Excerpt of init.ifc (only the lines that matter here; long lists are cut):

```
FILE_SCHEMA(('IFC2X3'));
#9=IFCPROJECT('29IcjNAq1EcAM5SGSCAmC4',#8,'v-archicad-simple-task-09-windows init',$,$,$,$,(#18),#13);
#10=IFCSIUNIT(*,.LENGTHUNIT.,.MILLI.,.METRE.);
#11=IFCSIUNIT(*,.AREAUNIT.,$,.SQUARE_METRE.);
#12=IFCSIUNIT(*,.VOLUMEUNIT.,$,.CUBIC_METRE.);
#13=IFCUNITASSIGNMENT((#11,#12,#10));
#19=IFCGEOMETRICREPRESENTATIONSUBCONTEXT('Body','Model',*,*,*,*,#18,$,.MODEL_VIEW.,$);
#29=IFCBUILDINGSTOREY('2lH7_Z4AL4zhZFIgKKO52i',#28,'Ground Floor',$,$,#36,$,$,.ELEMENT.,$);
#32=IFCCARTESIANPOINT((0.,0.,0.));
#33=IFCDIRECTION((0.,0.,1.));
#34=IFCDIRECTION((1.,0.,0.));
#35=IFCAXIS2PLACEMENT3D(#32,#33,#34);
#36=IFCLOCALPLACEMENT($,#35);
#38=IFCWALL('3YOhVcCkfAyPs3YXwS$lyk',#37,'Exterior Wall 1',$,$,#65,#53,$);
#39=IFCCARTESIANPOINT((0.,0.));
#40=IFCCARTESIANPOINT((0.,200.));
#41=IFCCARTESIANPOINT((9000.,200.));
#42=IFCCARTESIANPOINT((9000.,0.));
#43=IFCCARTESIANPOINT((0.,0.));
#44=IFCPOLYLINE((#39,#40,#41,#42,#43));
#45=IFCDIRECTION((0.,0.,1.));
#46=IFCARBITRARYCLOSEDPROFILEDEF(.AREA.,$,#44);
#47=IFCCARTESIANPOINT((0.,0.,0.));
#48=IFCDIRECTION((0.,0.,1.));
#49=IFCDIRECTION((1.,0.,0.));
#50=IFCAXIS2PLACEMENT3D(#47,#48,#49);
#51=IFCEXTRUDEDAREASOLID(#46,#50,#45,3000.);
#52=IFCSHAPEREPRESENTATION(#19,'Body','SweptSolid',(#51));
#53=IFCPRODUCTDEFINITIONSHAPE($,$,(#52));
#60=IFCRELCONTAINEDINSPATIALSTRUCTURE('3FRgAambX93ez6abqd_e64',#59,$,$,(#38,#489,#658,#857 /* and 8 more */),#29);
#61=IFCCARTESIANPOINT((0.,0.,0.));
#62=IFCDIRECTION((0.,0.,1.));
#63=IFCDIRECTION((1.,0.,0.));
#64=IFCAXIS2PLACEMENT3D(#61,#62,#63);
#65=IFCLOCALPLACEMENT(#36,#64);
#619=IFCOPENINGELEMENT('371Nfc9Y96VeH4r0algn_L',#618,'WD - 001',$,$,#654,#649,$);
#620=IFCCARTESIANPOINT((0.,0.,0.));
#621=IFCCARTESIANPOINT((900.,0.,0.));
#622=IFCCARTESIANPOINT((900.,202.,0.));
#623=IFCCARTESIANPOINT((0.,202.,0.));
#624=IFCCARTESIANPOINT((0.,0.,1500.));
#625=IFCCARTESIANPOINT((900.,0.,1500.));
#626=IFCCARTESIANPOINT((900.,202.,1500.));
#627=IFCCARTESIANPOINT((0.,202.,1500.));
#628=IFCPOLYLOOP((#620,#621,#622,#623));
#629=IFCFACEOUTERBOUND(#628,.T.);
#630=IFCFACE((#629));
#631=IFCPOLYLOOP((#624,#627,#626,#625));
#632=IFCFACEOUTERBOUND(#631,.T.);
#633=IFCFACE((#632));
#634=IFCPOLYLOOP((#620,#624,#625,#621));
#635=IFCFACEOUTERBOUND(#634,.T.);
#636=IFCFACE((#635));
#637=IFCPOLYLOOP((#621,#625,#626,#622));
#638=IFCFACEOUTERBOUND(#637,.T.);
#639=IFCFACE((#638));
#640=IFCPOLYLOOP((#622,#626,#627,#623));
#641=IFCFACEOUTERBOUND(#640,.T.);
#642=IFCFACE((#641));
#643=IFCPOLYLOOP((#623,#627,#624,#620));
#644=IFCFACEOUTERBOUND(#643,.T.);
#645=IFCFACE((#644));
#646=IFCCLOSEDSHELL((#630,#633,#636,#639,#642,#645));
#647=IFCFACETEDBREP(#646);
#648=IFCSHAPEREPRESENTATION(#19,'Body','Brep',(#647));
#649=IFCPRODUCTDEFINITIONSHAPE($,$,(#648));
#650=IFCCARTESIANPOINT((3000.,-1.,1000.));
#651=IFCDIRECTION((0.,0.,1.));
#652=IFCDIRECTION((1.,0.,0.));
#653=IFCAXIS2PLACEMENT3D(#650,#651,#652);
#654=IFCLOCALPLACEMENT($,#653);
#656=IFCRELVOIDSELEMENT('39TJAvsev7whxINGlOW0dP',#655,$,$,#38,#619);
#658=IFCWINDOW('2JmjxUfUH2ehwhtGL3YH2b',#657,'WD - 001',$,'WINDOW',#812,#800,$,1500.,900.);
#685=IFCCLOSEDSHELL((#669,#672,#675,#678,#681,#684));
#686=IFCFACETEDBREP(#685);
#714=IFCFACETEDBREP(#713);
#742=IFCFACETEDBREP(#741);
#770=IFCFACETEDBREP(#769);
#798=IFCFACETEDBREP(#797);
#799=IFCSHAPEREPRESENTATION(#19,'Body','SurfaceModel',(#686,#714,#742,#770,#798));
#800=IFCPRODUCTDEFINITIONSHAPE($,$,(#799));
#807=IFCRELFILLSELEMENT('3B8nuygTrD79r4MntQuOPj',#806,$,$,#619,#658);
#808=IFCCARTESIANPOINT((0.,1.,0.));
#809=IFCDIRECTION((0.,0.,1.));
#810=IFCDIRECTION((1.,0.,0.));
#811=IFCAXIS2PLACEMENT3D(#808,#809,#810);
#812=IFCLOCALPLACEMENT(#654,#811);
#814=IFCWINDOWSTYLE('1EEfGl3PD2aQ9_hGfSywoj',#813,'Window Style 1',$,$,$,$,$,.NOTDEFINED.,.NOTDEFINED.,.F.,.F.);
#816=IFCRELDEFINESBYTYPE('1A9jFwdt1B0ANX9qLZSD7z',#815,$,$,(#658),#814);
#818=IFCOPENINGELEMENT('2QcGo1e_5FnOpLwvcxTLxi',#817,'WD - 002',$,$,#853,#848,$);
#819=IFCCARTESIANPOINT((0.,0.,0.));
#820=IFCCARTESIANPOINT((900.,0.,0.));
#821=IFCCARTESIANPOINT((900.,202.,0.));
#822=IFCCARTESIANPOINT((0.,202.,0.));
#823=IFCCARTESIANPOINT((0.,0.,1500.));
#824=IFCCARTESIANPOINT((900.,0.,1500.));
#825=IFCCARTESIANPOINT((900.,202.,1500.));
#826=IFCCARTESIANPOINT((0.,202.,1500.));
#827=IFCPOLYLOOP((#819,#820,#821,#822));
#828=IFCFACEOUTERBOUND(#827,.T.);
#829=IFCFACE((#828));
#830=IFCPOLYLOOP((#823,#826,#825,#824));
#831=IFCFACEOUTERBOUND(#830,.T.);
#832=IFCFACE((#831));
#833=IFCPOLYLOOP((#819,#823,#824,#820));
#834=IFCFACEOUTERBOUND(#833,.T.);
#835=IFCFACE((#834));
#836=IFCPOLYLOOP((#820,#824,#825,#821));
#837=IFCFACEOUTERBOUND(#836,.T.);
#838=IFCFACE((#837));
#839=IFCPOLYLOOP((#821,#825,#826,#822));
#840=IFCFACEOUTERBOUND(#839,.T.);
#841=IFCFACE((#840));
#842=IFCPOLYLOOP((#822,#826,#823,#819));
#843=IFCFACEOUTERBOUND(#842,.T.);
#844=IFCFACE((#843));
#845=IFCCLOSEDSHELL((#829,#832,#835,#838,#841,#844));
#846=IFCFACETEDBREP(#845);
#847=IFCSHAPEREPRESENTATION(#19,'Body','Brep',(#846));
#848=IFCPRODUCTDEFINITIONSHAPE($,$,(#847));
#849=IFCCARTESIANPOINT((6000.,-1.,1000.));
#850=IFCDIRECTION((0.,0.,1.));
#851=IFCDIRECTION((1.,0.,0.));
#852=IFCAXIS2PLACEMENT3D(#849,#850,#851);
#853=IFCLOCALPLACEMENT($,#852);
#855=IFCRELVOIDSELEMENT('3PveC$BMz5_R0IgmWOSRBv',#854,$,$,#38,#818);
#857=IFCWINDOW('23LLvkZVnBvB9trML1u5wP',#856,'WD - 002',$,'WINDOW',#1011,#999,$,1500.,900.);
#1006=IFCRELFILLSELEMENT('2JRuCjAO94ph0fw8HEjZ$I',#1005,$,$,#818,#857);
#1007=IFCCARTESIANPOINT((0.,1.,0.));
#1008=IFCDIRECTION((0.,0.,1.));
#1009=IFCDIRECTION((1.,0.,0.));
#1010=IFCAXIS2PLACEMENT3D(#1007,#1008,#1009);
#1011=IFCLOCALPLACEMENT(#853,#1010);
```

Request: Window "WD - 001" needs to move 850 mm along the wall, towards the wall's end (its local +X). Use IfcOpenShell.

```python
import ifcopenshell
import ifcopenshell.api.geometry
import ifcopenshell.util.placement

model = ifcopenshell.open("init.ifc")

window = model.by_guid("2JmjxUfUH2ehwhtGL3YH2b")
opening = window.FillsVoids[0].RelatingOpeningElement
wall = opening.VoidsElements[0].RelatingBuildingElement

wall_matrix = ifcopenshell.util.placement.get_local_placement(wall.ObjectPlacement)
shift = wall_matrix[:3, 0] * 850.0
before = ifcopenshell.util.placement.get_local_placement(window.ObjectPlacement)[:3, 3].copy()

# The window is placed relative to its opening, so it follows when the opening moves.
matrix = ifcopenshell.util.placement.get_local_placement(opening.ObjectPlacement)
matrix[:3, 3] += shift
ifcopenshell.api.geometry.edit_object_placement(
    model, product=opening, matrix=matrix, is_si=False, should_transform_children=True
)

after = ifcopenshell.util.placement.get_local_placement(window.ObjectPlacement)[:3, 3]
print("window moved by", (after - before).round(3) + 0.0)

model.write("init_rev.ifc")
```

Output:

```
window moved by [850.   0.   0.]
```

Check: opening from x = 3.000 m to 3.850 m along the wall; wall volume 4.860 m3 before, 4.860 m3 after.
